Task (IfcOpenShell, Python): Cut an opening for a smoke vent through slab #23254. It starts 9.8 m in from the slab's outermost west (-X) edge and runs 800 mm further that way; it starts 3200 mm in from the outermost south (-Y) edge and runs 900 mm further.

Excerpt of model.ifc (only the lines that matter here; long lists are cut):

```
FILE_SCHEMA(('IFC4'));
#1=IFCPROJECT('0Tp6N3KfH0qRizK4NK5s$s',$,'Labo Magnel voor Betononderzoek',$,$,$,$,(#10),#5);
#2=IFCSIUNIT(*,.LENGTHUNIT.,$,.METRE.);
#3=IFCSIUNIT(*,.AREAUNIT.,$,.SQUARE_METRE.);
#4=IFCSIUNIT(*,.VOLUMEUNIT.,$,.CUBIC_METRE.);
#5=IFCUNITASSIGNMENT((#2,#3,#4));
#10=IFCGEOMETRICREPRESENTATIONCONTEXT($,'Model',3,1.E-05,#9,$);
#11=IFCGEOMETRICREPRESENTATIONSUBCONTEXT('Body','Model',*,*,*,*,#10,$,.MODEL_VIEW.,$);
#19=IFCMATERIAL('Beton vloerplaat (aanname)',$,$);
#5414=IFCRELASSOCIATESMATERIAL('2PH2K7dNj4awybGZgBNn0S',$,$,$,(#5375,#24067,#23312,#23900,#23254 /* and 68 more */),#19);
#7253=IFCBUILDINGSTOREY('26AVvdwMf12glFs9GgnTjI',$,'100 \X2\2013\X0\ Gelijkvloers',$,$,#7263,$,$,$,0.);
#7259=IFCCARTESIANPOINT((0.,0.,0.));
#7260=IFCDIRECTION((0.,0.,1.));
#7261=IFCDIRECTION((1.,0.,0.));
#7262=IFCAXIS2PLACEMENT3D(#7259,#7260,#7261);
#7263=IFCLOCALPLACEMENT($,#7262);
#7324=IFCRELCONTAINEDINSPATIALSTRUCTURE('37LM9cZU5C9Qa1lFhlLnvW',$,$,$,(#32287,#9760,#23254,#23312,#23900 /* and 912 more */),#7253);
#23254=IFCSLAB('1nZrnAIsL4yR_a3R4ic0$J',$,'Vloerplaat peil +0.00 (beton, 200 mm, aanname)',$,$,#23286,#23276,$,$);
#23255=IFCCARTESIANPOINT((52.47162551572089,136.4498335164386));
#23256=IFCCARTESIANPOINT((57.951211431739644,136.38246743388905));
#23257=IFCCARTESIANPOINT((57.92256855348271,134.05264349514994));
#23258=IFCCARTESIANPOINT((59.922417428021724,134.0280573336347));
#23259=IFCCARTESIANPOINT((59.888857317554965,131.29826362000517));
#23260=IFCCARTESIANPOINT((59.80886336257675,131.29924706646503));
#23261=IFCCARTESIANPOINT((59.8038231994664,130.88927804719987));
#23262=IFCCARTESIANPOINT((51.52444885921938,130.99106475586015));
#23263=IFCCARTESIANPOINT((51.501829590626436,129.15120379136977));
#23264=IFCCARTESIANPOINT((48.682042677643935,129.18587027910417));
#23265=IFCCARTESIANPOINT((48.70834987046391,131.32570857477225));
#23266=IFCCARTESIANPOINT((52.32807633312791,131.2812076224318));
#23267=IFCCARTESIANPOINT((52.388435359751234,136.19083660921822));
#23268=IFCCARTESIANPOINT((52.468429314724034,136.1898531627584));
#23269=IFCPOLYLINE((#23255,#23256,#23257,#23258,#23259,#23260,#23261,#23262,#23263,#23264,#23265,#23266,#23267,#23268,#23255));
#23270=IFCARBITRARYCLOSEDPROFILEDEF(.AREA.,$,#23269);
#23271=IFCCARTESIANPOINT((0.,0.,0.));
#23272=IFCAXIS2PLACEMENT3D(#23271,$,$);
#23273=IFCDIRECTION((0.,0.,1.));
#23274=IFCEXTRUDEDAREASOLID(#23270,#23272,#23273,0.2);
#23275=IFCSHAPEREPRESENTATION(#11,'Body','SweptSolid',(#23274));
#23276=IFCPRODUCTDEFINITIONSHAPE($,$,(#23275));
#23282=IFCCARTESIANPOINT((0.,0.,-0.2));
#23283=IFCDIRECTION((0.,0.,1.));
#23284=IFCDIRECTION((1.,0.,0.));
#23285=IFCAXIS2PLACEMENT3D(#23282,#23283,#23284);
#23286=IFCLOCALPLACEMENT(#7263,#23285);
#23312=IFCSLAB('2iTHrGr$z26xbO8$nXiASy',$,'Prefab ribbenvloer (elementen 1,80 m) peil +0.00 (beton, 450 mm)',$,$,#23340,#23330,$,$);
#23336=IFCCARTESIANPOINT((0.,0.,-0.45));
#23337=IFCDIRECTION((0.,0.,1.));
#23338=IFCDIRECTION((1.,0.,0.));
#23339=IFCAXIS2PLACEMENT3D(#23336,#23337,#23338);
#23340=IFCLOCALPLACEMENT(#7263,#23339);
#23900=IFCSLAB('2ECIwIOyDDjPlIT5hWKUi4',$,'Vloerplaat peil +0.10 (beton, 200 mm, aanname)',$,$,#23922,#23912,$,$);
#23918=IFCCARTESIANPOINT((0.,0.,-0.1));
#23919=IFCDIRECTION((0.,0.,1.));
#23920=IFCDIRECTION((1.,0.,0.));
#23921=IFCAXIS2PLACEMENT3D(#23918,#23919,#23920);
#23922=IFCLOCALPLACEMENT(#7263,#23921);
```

```python
import numpy as np
import ifcopenshell
import ifcopenshell.api.feature
import ifcopenshell.api.geometry
import ifcopenshell.api.root
import ifcopenshell.geom
import ifcopenshell.util.placement
import ifcopenshell.util.representation
import ifcopenshell.util.shape
import ifcopenshell.util.unit

model = ifcopenshell.open("model.ifc")
unit_scale = ifcopenshell.util.unit.calculate_unit_scale(model)
settings = ifcopenshell.geom.settings()


def volume(element):
    """Net volume in cubic metres, openings subtracted."""
    shape = ifcopenshell.geom.create_shape(settings, element)
    return ifcopenshell.util.shape.get_volume(shape.geometry)


slab = model.by_guid("1nZrnAIsL4yR_a3R4ic0$J")
before = volume(slab)

# Extent in the slab's own axes, in metres. The edges named are its -X and -Y sides.
slab_shape = ifcopenshell.geom.create_shape(settings, slab)
vertices = ifcopenshell.util.shape.get_vertices(slab_shape.geometry)
x_min, y_min, bottom = vertices.min(axis=0)
top = vertices[:, 2].max()

opening = ifcopenshell.api.root.create_entity(model, ifc_class="IfcOpeningElement", name="Smoke vent opening", predefined_type="OPENING")
context = ifcopenshell.util.representation.get_context(model, "Model", "Body", "MODEL_VIEW")
width, depth = 0.8, 0.9
outline = [(0.0, 0.0), (width, 0.0), (width, depth), (0.0, depth), (0.0, 0.0)]
# Overshoot both faces by 50 mm so the cut is clean.
shape = ifcopenshell.api.geometry.add_slab_representation(
    model, context=context, depth=top - bottom + 0.1, polyline=outline
)
ifcopenshell.api.geometry.assign_representation(model, product=opening, representation=shape)

matrix = ifcopenshell.util.placement.get_local_placement(slab.ObjectPlacement)
matrix[:, 3] = matrix @ np.append(np.array([x_min + 9.8, y_min + 3.2, bottom - 0.05]) / unit_scale, 1.0)
ifcopenshell.api.geometry.edit_object_placement(model, product=opening, matrix=matrix, is_si=False)
ifcopenshell.api.feature.add_feature(model, feature=opening, element=slab)

after = volume(slab)

print(f"slab volume {before:.3f} -> {after:.3f} m3")

model.write("model_updated.ifc")
```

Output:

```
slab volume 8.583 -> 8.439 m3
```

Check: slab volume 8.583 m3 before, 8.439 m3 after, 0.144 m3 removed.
